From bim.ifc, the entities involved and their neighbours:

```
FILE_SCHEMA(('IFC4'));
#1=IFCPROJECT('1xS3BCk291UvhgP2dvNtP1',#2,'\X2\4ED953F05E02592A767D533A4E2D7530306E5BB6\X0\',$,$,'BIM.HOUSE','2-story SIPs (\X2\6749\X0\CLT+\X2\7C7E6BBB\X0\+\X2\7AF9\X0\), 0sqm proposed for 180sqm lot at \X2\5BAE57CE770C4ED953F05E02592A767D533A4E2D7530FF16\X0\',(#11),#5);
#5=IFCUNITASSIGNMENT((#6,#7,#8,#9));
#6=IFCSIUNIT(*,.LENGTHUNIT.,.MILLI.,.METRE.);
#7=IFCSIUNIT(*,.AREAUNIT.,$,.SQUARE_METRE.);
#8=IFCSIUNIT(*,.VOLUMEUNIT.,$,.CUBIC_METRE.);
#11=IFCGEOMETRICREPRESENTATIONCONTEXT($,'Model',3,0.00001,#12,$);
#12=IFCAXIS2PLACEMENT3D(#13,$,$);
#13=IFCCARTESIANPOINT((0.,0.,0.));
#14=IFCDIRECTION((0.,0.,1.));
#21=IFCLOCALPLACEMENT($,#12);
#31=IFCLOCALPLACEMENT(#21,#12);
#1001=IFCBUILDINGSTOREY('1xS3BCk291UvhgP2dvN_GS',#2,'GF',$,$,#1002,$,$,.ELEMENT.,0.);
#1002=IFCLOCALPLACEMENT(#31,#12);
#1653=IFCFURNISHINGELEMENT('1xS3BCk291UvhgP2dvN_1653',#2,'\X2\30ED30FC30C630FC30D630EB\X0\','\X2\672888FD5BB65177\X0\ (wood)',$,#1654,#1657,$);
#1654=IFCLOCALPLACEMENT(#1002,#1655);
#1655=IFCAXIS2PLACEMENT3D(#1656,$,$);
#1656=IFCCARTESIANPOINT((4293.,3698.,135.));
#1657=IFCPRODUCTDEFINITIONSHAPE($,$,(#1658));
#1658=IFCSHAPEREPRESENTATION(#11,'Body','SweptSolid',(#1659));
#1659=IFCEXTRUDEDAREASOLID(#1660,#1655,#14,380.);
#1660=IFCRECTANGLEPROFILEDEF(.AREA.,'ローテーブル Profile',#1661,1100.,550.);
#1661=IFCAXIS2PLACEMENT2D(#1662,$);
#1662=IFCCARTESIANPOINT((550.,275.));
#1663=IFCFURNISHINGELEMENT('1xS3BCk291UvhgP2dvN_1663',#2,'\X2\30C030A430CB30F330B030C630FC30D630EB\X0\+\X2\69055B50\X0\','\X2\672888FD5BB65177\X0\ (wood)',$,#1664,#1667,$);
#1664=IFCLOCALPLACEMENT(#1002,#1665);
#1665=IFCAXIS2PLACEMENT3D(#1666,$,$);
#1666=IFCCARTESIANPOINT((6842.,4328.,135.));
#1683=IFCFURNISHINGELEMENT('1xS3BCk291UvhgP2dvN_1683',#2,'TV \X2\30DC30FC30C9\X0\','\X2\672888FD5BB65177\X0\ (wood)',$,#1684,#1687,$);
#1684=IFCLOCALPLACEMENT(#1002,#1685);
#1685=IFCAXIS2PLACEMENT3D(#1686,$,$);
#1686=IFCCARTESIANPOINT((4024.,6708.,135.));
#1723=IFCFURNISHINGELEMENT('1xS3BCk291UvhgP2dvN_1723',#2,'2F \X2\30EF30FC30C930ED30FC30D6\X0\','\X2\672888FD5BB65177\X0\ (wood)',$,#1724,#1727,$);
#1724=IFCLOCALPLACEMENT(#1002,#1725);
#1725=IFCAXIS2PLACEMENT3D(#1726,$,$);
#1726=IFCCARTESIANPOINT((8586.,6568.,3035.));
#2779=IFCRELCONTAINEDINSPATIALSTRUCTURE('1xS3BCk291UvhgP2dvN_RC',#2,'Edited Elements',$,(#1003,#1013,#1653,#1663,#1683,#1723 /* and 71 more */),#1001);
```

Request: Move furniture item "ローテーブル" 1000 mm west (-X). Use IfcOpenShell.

```python
import ifcopenshell
import ifcopenshell.api.geometry
import ifcopenshell.util.placement
import ifcopenshell.util.unit

model = ifcopenshell.open("bim.ifc")
unit_scale = ifcopenshell.util.unit.calculate_unit_scale(model)

item = model.by_id(1653)
matrix = ifcopenshell.util.placement.get_local_placement(item.ObjectPlacement)
matrix[0, 3] -= 1 / unit_scale
ifcopenshell.api.geometry.edit_object_placement(model, product=item, matrix=matrix, is_si=False)

print(ifcopenshell.util.placement.get_local_placement(item.ObjectPlacement).round(3) + 0.0)

model.write("bim_v2.ifc")
```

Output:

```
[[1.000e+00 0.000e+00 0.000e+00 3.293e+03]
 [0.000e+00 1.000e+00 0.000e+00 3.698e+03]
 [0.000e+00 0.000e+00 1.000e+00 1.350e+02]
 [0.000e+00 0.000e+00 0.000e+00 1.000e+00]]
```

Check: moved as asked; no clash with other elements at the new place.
